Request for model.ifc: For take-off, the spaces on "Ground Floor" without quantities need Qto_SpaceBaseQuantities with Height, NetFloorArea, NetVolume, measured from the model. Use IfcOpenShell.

First a look at what the model holds.

```python
import ifcopenshell
import ifcopenshell.util.element
import ifcopenshell.util.unit

model = ifcopenshell.open("model.ifc")
print(model.schema)
for unit_type in ("LENGTHUNIT", "AREAUNIT", "VOLUMEUNIT"):
    print(unit_type, ifcopenshell.util.unit.calculate_unit_scale(model, unit_type))
storey = next(s for s in model.by_type("IfcBuildingStorey") if s.Name == "Ground Floor")
spaces = [e for e in ifcopenshell.util.element.get_decomposition(storey) if e.is_a("IfcSpace")]
for e in sorted(spaces, key=lambda e: e.id()):
    print(e.id(), e.is_a(), e.Name, list(ifcopenshell.util.element.get_psets(e, qtos_only=True)), sep=" | ")
```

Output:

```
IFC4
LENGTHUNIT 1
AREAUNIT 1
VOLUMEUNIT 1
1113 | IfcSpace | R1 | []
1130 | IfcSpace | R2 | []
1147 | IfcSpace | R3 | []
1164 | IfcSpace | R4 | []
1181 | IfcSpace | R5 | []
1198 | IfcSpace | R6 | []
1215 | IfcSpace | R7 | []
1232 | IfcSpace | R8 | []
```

```python
import ifcopenshell
import ifcopenshell.api.pset
import ifcopenshell.geom
import ifcopenshell.util.element
import ifcopenshell.util.shape
import ifcopenshell.util.unit

model = ifcopenshell.open("model.ifc")
unit_scale = ifcopenshell.util.unit.calculate_unit_scale(model)
area_scale = ifcopenshell.util.unit.calculate_unit_scale(model, "AREAUNIT")
volume_scale = ifcopenshell.util.unit.calculate_unit_scale(model, "VOLUMEUNIT")
settings = ifcopenshell.geom.settings()

storey = next(s for s in model.by_type("IfcBuildingStorey") if s.Name == "Ground Floor")
spaces = [e for e in ifcopenshell.util.element.get_decomposition(storey) if e.is_a("IfcSpace")]

for e in sorted(spaces, key=lambda e: e.id()):
    if ifcopenshell.util.element.get_psets(e, qtos_only=True, should_inherit=False):
        continue
    # Geometry comes back in metres, in the element's own axes.
    shape = ifcopenshell.geom.create_shape(settings, e)
    values = {
        "Height": ifcopenshell.util.shape.get_z(shape.geometry) / unit_scale,
        "NetFloorArea": ifcopenshell.util.shape.get_footprint_area(shape.geometry) / area_scale,
        "NetVolume": ifcopenshell.util.shape.get_volume(shape.geometry) / volume_scale,
    }
    qto = ifcopenshell.api.pset.add_qto(model, product=e, name="Qto_SpaceBaseQuantities")
    ifcopenshell.api.pset.edit_qto(model, qto=qto, properties=values)
    print(e.id(), {k: round(v, 3) for k, v in values.items()})

model.write("model_updated.ifc")
```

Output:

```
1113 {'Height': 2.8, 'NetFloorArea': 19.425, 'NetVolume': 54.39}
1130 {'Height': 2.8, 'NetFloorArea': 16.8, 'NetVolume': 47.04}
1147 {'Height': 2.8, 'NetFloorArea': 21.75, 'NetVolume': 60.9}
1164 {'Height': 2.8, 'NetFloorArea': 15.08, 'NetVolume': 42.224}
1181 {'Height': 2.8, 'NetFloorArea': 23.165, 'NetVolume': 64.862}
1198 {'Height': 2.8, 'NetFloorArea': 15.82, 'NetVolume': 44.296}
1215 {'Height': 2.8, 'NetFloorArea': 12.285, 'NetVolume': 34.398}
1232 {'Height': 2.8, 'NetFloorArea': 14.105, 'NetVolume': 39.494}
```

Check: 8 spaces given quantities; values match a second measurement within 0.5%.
